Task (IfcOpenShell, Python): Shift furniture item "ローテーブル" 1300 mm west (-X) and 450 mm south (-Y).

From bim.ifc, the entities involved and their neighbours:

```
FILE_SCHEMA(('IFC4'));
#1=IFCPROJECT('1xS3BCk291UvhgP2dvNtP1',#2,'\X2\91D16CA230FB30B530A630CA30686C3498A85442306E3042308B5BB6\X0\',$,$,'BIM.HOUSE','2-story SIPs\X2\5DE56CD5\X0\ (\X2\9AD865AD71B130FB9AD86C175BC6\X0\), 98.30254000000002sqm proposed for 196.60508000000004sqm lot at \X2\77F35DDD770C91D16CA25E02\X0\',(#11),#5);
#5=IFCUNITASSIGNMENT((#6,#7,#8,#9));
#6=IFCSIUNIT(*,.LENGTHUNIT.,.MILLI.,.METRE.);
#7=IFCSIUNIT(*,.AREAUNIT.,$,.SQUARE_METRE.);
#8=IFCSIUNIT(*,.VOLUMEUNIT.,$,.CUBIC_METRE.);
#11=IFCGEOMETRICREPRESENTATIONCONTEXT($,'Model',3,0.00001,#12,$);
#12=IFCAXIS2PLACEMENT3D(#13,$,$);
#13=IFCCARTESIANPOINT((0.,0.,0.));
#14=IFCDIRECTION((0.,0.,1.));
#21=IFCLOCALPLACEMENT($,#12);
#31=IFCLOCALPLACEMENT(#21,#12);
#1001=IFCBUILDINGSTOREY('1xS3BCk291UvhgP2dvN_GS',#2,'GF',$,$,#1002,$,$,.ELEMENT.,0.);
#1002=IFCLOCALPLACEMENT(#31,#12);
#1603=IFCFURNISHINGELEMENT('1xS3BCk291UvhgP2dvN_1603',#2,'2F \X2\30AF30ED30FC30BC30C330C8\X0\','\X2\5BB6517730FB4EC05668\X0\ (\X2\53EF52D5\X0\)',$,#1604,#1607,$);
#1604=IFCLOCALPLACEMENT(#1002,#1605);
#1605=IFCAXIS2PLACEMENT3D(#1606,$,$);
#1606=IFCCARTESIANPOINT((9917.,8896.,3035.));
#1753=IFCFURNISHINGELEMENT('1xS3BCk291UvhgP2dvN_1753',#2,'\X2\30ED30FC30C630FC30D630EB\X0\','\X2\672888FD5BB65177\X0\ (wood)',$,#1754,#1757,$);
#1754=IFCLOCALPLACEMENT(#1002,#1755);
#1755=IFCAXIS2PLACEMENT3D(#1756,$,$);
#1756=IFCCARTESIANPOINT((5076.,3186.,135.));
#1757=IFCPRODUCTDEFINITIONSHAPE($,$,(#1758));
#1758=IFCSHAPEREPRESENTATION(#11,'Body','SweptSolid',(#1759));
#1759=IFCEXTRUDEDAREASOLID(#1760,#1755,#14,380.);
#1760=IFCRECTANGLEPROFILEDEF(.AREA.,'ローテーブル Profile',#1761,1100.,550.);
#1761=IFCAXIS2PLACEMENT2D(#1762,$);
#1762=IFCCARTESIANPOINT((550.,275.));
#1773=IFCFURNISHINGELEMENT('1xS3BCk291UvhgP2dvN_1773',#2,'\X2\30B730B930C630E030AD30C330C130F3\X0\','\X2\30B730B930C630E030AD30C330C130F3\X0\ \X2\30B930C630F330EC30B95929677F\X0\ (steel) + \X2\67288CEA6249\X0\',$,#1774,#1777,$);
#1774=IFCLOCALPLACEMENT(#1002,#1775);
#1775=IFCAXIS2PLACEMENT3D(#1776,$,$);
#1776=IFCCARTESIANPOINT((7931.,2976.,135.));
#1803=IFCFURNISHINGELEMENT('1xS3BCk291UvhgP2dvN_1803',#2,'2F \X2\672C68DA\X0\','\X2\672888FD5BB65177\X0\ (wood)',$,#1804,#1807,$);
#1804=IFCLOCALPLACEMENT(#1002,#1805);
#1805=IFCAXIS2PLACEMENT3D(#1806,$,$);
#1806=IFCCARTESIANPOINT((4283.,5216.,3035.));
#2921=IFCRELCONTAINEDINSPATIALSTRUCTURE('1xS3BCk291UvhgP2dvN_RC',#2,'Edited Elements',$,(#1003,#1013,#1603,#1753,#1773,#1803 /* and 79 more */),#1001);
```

```python
import ifcopenshell
import ifcopenshell.api.geometry
import ifcopenshell.util.placement

model = ifcopenshell.open("bim.ifc")

item = model.by_guid("1xS3BCk291UvhgP2dvN_1753")
matrix = ifcopenshell.util.placement.get_local_placement(item.ObjectPlacement)
matrix[0, 3] -= 1300.0
matrix[1, 3] -= 450.0
ifcopenshell.api.geometry.edit_object_placement(model, product=item, matrix=matrix, is_si=False)

print(ifcopenshell.util.placement.get_local_placement(item.ObjectPlacement).round(3) + 0.0)

model.write("bim_edited.ifc")
```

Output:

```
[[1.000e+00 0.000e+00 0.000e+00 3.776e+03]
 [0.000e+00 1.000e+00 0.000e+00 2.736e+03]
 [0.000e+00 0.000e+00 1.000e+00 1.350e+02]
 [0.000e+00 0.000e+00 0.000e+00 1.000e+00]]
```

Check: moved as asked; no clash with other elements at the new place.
